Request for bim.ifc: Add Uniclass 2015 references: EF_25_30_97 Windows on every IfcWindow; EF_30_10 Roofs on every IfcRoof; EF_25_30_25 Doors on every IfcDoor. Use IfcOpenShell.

First a look at what the model holds.

```python
import ifcopenshell

model = ifcopenshell.open("bim.ifc")
print(model.schema)
print("classifications:", [c.Name for c in model.by_type("IfcClassification")])
for ifc_class in ("IfcDoor", "IfcRoof", "IfcStair", "IfcWall", "IfcWindow"):
    print(ifc_class, len(model.by_type(ifc_class)))
```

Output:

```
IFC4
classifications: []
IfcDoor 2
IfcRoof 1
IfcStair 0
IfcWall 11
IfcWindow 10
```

```python
import ifcopenshell
import ifcopenshell.api.classification

model = ifcopenshell.open("bim.ifc")

system = ifcopenshell.api.classification.add_classification(model, classification="Uniclass 2015")

codes = {
    "IfcWindow": ("EF_25_30_97", "Windows"),
    "IfcRoof": ("EF_30_10", "Roofs"),
    "IfcDoor": ("EF_25_30_25", "Doors"),
}
for ifc_class, (code, name) in codes.items():
    products = model.by_type(ifc_class)
    ifcopenshell.api.classification.add_reference(
        model, products=products, classification=system, identification=code, name=name
    )
    print(code, len(products))

model.write("bim_edited.ifc")
```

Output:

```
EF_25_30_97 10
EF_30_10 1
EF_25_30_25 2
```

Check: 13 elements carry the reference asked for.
